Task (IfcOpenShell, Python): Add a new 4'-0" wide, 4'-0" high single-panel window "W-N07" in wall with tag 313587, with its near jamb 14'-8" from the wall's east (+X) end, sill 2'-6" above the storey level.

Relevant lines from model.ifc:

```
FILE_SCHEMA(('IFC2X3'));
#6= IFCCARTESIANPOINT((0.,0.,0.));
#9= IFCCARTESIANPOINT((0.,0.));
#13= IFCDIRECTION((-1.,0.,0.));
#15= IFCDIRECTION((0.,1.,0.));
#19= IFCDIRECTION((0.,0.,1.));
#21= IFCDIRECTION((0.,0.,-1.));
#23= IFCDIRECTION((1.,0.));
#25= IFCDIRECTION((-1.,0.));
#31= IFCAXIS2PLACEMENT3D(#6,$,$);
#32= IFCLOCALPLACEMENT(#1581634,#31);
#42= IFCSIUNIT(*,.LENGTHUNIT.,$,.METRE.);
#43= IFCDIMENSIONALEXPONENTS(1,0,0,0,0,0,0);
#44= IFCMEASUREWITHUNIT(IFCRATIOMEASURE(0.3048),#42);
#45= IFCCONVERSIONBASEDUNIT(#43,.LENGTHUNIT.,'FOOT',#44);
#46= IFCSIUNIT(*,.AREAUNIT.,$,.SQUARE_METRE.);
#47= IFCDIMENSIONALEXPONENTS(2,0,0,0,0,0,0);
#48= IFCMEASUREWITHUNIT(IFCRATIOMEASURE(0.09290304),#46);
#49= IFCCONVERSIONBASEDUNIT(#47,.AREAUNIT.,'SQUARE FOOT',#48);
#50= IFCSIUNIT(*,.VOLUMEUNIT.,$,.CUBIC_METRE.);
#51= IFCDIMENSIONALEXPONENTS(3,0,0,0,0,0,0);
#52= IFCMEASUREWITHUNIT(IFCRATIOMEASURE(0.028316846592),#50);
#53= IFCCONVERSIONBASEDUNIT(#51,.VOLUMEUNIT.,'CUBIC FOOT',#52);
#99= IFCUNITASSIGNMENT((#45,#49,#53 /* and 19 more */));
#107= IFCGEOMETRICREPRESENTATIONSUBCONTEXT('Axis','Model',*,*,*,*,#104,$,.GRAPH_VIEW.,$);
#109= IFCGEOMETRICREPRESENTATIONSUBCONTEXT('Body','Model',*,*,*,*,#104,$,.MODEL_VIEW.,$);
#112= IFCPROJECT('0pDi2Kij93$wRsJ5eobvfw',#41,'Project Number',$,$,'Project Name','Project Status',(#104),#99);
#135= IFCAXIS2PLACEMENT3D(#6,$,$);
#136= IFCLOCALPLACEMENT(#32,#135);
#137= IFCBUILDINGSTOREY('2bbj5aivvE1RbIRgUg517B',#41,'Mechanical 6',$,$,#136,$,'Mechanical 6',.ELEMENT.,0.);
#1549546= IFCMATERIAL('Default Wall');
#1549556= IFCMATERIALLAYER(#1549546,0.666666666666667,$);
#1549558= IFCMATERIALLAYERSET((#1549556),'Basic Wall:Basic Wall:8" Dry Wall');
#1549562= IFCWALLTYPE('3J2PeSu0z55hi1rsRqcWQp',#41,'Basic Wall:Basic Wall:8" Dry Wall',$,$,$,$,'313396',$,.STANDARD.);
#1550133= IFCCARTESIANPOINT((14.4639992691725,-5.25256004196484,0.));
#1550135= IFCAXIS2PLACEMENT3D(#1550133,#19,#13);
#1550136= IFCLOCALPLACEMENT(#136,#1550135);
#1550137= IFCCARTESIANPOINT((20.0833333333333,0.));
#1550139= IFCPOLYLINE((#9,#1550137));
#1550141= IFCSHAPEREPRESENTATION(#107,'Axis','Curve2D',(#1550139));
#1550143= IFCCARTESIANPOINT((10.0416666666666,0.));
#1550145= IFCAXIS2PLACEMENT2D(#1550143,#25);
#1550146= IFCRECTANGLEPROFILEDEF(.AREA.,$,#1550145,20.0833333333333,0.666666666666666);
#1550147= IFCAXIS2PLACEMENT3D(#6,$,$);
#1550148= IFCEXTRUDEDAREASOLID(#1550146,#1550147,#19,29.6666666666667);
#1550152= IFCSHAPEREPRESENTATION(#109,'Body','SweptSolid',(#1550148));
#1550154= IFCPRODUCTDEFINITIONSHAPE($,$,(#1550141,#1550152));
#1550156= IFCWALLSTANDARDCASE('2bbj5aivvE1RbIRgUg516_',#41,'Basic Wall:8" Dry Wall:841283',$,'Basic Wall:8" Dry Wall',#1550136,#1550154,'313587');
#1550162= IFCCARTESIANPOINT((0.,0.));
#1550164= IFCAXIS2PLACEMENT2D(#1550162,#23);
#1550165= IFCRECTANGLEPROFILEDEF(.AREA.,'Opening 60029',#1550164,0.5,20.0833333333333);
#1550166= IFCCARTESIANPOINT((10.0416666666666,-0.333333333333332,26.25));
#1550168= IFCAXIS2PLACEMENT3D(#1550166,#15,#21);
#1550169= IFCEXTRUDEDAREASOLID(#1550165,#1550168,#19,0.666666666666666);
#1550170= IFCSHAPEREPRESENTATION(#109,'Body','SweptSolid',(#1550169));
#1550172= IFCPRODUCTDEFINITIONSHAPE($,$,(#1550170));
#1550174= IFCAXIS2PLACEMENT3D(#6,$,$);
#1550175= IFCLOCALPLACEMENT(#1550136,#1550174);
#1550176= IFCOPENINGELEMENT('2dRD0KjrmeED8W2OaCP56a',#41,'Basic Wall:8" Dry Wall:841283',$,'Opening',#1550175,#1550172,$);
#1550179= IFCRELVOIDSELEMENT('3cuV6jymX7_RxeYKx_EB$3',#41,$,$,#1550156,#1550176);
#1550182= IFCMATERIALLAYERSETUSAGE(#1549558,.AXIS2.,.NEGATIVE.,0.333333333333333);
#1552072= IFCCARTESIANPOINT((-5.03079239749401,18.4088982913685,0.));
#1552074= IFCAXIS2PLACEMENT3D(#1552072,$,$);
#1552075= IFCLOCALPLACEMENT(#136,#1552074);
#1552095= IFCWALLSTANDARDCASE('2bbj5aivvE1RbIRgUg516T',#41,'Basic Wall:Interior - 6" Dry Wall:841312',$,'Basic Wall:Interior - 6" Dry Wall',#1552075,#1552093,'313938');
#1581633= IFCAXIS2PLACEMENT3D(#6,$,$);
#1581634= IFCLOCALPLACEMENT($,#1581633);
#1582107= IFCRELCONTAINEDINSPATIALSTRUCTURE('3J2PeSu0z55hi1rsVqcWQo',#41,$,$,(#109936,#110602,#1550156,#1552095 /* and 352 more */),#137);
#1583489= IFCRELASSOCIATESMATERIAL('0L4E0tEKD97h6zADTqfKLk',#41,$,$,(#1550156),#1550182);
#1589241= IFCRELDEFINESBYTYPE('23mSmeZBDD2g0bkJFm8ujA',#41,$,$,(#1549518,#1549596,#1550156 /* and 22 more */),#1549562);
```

```python
import numpy as np
import ifcopenshell
import ifcopenshell.api.feature
import ifcopenshell.api.geometry
import ifcopenshell.api.root
import ifcopenshell.api.spatial
import ifcopenshell.api.type
import ifcopenshell.geom
import ifcopenshell.util.element
import ifcopenshell.util.placement
import ifcopenshell.util.representation
import ifcopenshell.util.shape
import ifcopenshell.util.unit

model = ifcopenshell.open("model.ifc")
unit_scale = ifcopenshell.util.unit.calculate_unit_scale(model)
settings = ifcopenshell.geom.settings()


def volume(element):
    """Net volume in cubic metres, openings subtracted."""
    shape = ifcopenshell.geom.create_shape(settings, element)
    return ifcopenshell.util.shape.get_volume(shape.geometry)


wall = model.by_guid("2bbj5aivvE1RbIRgUg516_")
storey = ifcopenshell.util.element.get_container(wall, ifc_class="IfcBuildingStorey")
context = ifcopenshell.util.representation.get_context(model, "Model", "Body", "MODEL_VIEW")
before = volume(wall)

width, height, from_end, sill = 1.2192, 1.2192, 4.4704, 0.762  # metres

# The wall runs along its own X axis, and the end named is its -X end.
wall_shape = ifcopenshell.geom.create_shape(settings, wall)
x, y, z = ifcopenshell.util.shape.get_vertices(wall_shape.geometry).T
start = x.min() + from_end
face, thickness = float(y.min()), float(y.max() - y.min())
wall_matrix = ifcopenshell.util.placement.get_local_placement(wall.ObjectPlacement)
level = ifcopenshell.util.placement.get_local_placement(storey.ObjectPlacement)[2, 3]


def in_wall(x, y):
    """Placement at x, y metres in the wall's axes, at sill height."""
    matrix = wall_matrix.copy()
    matrix[:, 3] = wall_matrix @ np.array([x / unit_scale, y / unit_scale, 0.0, 1.0])
    matrix[2, 3] = level + sill / unit_scale
    return matrix


# Opening: a box that overshoots both wall faces by 50 mm.
opening = ifcopenshell.api.root.create_entity(model, ifc_class="IfcOpeningElement")
box = ifcopenshell.api.geometry.add_wall_representation(
    model, context=context, length=width, height=height, thickness=thickness + 0.1
)
ifcopenshell.api.geometry.assign_representation(model, product=opening, representation=box)
ifcopenshell.api.geometry.edit_object_placement(model, product=opening, matrix=in_wall(start, face - 0.05), is_si=False)
ifcopenshell.api.feature.add_feature(model, feature=opening, element=wall)

window = ifcopenshell.api.root.create_entity(model, ifc_class="IfcWindow", name="W-N07")
window.OverallWidth, window.OverallHeight = width / unit_scale, height / unit_scale
body = ifcopenshell.api.geometry.add_window_representation(
    model,
    context=context,
    overall_width=window.OverallWidth,
    overall_height=window.OverallHeight,
    partition_type="SINGLE_PANEL",
)
ifcopenshell.api.geometry.assign_representation(model, product=window, representation=body)
ifcopenshell.api.spatial.assign_container(model, products=[window], relating_structure=storey)
fills = ifcopenshell.api.feature.add_filling(model, opening=opening, element=window)
fills.OwnerHistory = window.OwnerHistory  # required in IFC2X3

# IFC2X3 keeps the operation on the window style.
style = ifcopenshell.api.root.create_entity(model, ifc_class="IfcWindowStyle", name="W-N07")
style.OperationType, style.ConstructionType = "SINGLE_PANEL", "NOTDEFINED"
style.ParameterTakesPrecedence = style.Sizeable = False
ifcopenshell.api.type.assign_type(model, related_objects=[window], relating_type=style)

# Centre the window in the wall's thickness.
ifcopenshell.api.geometry.edit_object_placement(model, product=window, matrix=in_wall(start, face), is_si=False)
window_shape = ifcopenshell.geom.create_shape(settings, window)
depth = ifcopenshell.util.shape.get_vertices(window_shape.geometry)[:, 1]
offset = face + thickness / 2 - (depth.min() + depth.max()) / 2
ifcopenshell.api.geometry.edit_object_placement(model, product=window, matrix=in_wall(start, offset), is_si=False)

after = volume(wall)

print(f"wall volume {before:.3f} -> {after:.3f} m3")

model.write("model_rev.ifc")
```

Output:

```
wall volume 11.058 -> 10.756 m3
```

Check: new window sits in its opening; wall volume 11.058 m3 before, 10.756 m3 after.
